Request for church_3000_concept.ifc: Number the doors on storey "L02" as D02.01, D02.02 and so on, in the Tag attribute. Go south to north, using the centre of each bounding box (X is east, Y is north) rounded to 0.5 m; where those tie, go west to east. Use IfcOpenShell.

First a look at what the model holds.

```python
import ifcopenshell
import ifcopenshell.util.element
import ifcopenshell.util.placement

model = ifcopenshell.open("church_3000_concept.ifc")
print(model.schema)
storey = next(s for s in model.by_type("IfcBuildingStorey") if s.Name == "L02")
doors = [e for e in ifcopenshell.util.element.get_decomposition(storey) if e.is_a("IfcDoor")]
for e in sorted(doors, key=lambda e: e.id()):
    origin = ifcopenshell.util.placement.get_local_placement(e.ObjectPlacement)[:3, 3]
    print(e.id(), e.Tag, e.Name, origin.round(2) + 0.0, sep=" | ")
```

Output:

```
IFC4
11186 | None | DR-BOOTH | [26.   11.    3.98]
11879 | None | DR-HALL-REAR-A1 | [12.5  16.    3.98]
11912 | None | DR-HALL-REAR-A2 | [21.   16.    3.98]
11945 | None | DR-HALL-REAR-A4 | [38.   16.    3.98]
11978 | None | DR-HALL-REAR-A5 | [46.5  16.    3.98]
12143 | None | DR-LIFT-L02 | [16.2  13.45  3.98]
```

```python
import ifcopenshell
import ifcopenshell.geom
import ifcopenshell.util.element
import ifcopenshell.util.shape

model = ifcopenshell.open("church_3000_concept.ifc")
settings = ifcopenshell.geom.settings()
settings.set("use-world-coords", True)


def centre(element):
    shape = ifcopenshell.geom.create_shape(settings, element)
    return ifcopenshell.util.shape.get_bbox_centroid(shape.geometry)


storey = next(s for s in model.by_type("IfcBuildingStorey") if s.Name == "L02")
doors = [e for e in ifcopenshell.util.element.get_decomposition(storey) if e.is_a("IfcDoor")]

# Insertion points can sit at a corner or the storey origin, so sort by the geometry (in metres).
centres = {e: centre(e) for e in doors}
doors.sort(key=lambda e: (round(centres[e][1] / 0.5), centres[e][0]))

for i, e in enumerate(doors, start=1):
    number = f"D02.{i:02d}"
    e.Tag = number
    print(e.id(), number)

model.write("church_3000_concept-out.ifc")
```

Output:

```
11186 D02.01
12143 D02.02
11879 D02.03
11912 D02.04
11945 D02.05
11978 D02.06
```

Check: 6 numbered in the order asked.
